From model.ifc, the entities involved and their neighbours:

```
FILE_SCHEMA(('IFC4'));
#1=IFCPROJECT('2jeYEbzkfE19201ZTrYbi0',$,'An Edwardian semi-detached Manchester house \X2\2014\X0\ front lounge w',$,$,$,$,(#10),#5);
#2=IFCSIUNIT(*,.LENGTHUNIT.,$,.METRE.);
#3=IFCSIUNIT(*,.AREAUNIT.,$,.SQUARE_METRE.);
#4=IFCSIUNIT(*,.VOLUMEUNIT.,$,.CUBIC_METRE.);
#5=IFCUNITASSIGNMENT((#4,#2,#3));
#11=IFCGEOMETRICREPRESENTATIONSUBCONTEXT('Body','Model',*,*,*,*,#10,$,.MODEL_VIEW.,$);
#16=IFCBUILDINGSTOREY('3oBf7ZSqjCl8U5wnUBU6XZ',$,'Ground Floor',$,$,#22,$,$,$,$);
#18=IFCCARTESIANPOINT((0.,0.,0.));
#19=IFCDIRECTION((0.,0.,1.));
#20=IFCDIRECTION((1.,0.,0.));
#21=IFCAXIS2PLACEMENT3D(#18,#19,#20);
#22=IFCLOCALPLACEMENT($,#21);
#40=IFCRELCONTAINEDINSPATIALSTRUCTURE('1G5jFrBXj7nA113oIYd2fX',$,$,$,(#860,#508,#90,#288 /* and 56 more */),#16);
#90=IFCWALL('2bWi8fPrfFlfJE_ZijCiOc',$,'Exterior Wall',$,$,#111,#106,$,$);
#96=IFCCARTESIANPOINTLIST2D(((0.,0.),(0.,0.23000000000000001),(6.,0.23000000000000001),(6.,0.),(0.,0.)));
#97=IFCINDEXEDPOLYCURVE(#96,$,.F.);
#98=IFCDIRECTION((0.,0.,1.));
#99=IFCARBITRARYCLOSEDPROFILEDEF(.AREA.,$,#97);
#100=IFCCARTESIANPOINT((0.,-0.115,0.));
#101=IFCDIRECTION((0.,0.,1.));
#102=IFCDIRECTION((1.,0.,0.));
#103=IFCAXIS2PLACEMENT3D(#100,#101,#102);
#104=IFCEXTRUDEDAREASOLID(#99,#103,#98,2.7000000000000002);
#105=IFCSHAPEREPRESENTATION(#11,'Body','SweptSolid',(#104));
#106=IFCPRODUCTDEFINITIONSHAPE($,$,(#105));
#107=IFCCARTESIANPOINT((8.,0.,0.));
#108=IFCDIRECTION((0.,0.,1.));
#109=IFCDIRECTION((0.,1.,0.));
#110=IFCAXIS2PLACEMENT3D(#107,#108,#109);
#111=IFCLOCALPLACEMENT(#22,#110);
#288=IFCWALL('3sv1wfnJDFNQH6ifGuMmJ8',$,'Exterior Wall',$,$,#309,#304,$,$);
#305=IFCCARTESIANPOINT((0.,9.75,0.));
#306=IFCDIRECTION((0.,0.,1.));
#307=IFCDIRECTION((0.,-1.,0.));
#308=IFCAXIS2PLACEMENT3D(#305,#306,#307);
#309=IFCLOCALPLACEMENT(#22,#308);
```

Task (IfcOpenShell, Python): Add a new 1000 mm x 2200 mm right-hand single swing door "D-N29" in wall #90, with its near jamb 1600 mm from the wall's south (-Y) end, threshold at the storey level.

```python
import numpy as np
import ifcopenshell
import ifcopenshell.api.feature
import ifcopenshell.api.geometry
import ifcopenshell.api.root
import ifcopenshell.api.spatial
import ifcopenshell.geom
import ifcopenshell.util.element
import ifcopenshell.util.placement
import ifcopenshell.util.representation
import ifcopenshell.util.shape
import ifcopenshell.util.unit

model = ifcopenshell.open("model.ifc")
unit_scale = ifcopenshell.util.unit.calculate_unit_scale(model)
settings = ifcopenshell.geom.settings()


def volume(element):
    """Net volume in cubic metres, openings subtracted."""
    shape = ifcopenshell.geom.create_shape(settings, element)
    return ifcopenshell.util.shape.get_volume(shape.geometry)


wall = model.by_guid("2bWi8fPrfFlfJE_ZijCiOc")
storey = ifcopenshell.util.element.get_container(wall, ifc_class="IfcBuildingStorey")
context = ifcopenshell.util.representation.get_context(model, "Model", "Body", "MODEL_VIEW")
before = volume(wall)

width, height, from_end, sill = 1, 2.2, 1.6, 0.0  # metres

# The wall runs along its own X axis, and the end named is its -X end.
wall_shape = ifcopenshell.geom.create_shape(settings, wall)
x, y, z = ifcopenshell.util.shape.get_vertices(wall_shape.geometry).T
start = x.min() + from_end
face, thickness = float(y.min()), float(y.max() - y.min())
wall_matrix = ifcopenshell.util.placement.get_local_placement(wall.ObjectPlacement)
level = ifcopenshell.util.placement.get_local_placement(storey.ObjectPlacement)[2, 3]


def in_wall(x, y):
    """Placement at x, y metres in the wall's axes, at sill height."""
    matrix = wall_matrix.copy()
    matrix[:, 3] = wall_matrix @ np.array([x / unit_scale, y / unit_scale, 0.0, 1.0])
    matrix[2, 3] = level + sill / unit_scale
    return matrix


# Opening: a box that overshoots both wall faces by 50 mm.
opening = ifcopenshell.api.root.create_entity(model, ifc_class="IfcOpeningElement", predefined_type="OPENING")
box = ifcopenshell.api.geometry.add_wall_representation(
    model, context=context, length=width, height=height, thickness=thickness + 0.1
)
ifcopenshell.api.geometry.assign_representation(model, product=opening, representation=box)
ifcopenshell.api.geometry.edit_object_placement(model, product=opening, matrix=in_wall(start, face - 0.05), is_si=False)
ifcopenshell.api.feature.add_feature(model, feature=opening, element=wall)

door = ifcopenshell.api.root.create_entity(model, ifc_class="IfcDoor", name="D-N29", predefined_type="DOOR")
door.OverallWidth, door.OverallHeight = width / unit_scale, height / unit_scale
door.OperationType = "SINGLE_SWING_RIGHT"
body = ifcopenshell.api.geometry.add_door_representation(
    model,
    context=context,
    overall_width=door.OverallWidth,
    overall_height=door.OverallHeight,
    operation_type="SINGLE_SWING_RIGHT",
    lining_properties={"LiningDepth": thickness / unit_scale, "ThresholdDepth": thickness / unit_scale},
)
ifcopenshell.api.geometry.assign_representation(model, product=door, representation=body)
ifcopenshell.api.spatial.assign_container(model, products=[door], relating_structure=storey)
ifcopenshell.api.feature.add_filling(model, opening=opening, element=door)

# The lining spans the wall, so the door starts at the wall face.
ifcopenshell.api.geometry.edit_object_placement(model, product=door, matrix=in_wall(start, face), is_si=False)

after = volume(wall)

print(f"wall volume {before:.3f} -> {after:.3f} m3")

model.write("model_edited.ifc")
```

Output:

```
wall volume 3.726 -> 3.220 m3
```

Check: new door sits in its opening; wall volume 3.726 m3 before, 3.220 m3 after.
